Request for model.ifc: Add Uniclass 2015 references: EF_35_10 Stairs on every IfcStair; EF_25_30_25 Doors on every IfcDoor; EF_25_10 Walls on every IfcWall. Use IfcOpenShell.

First a look at what the model holds.

```python
import ifcopenshell

model = ifcopenshell.open("model.ifc")
print(model.schema)
print("classifications:", [c.Name for c in model.by_type("IfcClassification")])
for ifc_class in ("IfcDoor", "IfcRoof", "IfcStair", "IfcWall", "IfcWindow"):
    print(ifc_class, len(model.by_type(ifc_class)))
```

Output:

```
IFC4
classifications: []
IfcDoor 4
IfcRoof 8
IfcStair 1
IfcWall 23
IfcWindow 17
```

```python
import ifcopenshell
import ifcopenshell.api.classification

model = ifcopenshell.open("model.ifc")

system = ifcopenshell.api.classification.add_classification(model, classification="Uniclass 2015")

codes = {
    "IfcStair": ("EF_35_10", "Stairs"),
    "IfcDoor": ("EF_25_30_25", "Doors"),
    "IfcWall": ("EF_25_10", "Walls"),
}
for ifc_class, (code, name) in codes.items():
    products = model.by_type(ifc_class)
    ifcopenshell.api.classification.add_reference(
        model, products=products, classification=system, identification=code, name=name
    )
    print(code, len(products))

model.write("model-out.ifc")
```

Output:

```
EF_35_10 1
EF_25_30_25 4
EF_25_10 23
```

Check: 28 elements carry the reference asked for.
